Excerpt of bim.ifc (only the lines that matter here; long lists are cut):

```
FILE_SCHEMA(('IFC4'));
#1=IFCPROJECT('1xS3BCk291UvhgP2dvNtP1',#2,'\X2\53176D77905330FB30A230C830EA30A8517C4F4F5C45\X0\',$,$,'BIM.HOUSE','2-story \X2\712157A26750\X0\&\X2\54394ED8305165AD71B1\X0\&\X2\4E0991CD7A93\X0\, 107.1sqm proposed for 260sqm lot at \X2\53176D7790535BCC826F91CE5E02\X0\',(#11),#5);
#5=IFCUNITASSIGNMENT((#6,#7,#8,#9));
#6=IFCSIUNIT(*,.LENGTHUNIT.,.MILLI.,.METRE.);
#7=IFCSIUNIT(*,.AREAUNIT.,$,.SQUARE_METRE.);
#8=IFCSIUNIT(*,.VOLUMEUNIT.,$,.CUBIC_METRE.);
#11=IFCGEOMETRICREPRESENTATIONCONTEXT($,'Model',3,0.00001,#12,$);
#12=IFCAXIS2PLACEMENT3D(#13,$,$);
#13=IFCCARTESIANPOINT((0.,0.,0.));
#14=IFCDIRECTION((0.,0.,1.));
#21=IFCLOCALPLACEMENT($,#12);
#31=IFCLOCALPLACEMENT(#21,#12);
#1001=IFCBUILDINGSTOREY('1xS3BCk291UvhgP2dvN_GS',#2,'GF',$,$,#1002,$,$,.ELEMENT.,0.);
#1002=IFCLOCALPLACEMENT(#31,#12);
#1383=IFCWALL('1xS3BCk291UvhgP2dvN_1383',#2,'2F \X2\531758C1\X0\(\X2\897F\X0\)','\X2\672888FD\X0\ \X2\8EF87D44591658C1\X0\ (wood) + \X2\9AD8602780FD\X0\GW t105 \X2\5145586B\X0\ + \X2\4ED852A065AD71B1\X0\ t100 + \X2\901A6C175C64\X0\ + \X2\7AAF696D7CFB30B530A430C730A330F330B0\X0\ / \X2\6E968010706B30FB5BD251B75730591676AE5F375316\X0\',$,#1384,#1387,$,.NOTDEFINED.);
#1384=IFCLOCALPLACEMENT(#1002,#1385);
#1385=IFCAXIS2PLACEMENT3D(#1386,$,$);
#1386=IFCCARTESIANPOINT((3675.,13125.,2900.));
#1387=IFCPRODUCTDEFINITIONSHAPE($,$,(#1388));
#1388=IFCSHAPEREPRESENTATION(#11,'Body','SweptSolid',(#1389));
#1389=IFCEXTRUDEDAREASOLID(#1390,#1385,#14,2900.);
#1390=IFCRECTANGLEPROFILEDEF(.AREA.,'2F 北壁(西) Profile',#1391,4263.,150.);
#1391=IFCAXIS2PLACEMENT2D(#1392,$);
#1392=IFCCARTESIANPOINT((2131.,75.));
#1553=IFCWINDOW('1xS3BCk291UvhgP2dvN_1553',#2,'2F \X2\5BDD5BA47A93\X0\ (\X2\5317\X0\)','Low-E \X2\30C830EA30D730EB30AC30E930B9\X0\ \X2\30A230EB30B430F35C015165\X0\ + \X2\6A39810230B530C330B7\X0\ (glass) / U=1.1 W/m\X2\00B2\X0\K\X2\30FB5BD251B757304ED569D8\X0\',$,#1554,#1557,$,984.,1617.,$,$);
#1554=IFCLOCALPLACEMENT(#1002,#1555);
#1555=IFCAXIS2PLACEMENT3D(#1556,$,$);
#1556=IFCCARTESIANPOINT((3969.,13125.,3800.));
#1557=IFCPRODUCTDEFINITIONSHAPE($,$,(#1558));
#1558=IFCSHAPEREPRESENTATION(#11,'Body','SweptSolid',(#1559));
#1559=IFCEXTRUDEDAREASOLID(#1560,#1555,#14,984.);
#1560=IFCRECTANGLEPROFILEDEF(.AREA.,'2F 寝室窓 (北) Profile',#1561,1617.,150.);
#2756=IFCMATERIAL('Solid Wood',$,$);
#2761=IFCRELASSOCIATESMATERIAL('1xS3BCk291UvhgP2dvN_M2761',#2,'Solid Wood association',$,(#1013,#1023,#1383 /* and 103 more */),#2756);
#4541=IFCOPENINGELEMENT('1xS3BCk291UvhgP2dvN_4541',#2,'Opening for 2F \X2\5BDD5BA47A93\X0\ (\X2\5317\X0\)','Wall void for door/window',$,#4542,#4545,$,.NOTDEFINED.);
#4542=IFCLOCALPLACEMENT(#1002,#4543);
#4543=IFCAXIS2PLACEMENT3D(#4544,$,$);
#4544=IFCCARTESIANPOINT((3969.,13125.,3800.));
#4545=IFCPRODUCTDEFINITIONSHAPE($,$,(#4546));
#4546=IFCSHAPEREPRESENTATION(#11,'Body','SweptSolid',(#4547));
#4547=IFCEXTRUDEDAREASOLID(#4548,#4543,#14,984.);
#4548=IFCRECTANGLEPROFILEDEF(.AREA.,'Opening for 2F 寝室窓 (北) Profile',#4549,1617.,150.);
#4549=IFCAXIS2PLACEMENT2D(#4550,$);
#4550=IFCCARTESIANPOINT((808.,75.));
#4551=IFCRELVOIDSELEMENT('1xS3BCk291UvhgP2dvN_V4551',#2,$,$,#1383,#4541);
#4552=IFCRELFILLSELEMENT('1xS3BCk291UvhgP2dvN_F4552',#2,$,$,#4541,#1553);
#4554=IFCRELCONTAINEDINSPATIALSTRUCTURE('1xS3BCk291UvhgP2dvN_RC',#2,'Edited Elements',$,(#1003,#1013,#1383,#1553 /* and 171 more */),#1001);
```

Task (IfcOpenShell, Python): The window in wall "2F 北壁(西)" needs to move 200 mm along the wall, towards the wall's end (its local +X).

```python
import ifcopenshell
import ifcopenshell.api.geometry
import ifcopenshell.util.placement
import ifcopenshell.util.unit

model = ifcopenshell.open("bim.ifc")
unit_scale = ifcopenshell.util.unit.calculate_unit_scale(model)

window = model.by_guid("1xS3BCk291UvhgP2dvN_1553")
opening = window.FillsVoids[0].RelatingOpeningElement
wall = opening.VoidsElements[0].RelatingBuildingElement

wall_matrix = ifcopenshell.util.placement.get_local_placement(wall.ObjectPlacement)
shift = wall_matrix[:3, 0] * 0.2 / unit_scale
before = ifcopenshell.util.placement.get_local_placement(window.ObjectPlacement)[:3, 3].copy()

# The window is not placed relative to its opening, so move both.
for product in (opening, window):
    matrix = ifcopenshell.util.placement.get_local_placement(product.ObjectPlacement)
    matrix[:3, 3] += shift
    ifcopenshell.api.geometry.edit_object_placement(model, product=product, matrix=matrix, is_si=False)

after = ifcopenshell.util.placement.get_local_placement(window.ObjectPlacement)[:3, 3]
print("window moved by", (after - before).round(3) + 0.0)

model.write("bim_v2.ifc")
```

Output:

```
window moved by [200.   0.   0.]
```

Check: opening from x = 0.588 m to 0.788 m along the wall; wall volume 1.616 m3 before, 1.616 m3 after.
